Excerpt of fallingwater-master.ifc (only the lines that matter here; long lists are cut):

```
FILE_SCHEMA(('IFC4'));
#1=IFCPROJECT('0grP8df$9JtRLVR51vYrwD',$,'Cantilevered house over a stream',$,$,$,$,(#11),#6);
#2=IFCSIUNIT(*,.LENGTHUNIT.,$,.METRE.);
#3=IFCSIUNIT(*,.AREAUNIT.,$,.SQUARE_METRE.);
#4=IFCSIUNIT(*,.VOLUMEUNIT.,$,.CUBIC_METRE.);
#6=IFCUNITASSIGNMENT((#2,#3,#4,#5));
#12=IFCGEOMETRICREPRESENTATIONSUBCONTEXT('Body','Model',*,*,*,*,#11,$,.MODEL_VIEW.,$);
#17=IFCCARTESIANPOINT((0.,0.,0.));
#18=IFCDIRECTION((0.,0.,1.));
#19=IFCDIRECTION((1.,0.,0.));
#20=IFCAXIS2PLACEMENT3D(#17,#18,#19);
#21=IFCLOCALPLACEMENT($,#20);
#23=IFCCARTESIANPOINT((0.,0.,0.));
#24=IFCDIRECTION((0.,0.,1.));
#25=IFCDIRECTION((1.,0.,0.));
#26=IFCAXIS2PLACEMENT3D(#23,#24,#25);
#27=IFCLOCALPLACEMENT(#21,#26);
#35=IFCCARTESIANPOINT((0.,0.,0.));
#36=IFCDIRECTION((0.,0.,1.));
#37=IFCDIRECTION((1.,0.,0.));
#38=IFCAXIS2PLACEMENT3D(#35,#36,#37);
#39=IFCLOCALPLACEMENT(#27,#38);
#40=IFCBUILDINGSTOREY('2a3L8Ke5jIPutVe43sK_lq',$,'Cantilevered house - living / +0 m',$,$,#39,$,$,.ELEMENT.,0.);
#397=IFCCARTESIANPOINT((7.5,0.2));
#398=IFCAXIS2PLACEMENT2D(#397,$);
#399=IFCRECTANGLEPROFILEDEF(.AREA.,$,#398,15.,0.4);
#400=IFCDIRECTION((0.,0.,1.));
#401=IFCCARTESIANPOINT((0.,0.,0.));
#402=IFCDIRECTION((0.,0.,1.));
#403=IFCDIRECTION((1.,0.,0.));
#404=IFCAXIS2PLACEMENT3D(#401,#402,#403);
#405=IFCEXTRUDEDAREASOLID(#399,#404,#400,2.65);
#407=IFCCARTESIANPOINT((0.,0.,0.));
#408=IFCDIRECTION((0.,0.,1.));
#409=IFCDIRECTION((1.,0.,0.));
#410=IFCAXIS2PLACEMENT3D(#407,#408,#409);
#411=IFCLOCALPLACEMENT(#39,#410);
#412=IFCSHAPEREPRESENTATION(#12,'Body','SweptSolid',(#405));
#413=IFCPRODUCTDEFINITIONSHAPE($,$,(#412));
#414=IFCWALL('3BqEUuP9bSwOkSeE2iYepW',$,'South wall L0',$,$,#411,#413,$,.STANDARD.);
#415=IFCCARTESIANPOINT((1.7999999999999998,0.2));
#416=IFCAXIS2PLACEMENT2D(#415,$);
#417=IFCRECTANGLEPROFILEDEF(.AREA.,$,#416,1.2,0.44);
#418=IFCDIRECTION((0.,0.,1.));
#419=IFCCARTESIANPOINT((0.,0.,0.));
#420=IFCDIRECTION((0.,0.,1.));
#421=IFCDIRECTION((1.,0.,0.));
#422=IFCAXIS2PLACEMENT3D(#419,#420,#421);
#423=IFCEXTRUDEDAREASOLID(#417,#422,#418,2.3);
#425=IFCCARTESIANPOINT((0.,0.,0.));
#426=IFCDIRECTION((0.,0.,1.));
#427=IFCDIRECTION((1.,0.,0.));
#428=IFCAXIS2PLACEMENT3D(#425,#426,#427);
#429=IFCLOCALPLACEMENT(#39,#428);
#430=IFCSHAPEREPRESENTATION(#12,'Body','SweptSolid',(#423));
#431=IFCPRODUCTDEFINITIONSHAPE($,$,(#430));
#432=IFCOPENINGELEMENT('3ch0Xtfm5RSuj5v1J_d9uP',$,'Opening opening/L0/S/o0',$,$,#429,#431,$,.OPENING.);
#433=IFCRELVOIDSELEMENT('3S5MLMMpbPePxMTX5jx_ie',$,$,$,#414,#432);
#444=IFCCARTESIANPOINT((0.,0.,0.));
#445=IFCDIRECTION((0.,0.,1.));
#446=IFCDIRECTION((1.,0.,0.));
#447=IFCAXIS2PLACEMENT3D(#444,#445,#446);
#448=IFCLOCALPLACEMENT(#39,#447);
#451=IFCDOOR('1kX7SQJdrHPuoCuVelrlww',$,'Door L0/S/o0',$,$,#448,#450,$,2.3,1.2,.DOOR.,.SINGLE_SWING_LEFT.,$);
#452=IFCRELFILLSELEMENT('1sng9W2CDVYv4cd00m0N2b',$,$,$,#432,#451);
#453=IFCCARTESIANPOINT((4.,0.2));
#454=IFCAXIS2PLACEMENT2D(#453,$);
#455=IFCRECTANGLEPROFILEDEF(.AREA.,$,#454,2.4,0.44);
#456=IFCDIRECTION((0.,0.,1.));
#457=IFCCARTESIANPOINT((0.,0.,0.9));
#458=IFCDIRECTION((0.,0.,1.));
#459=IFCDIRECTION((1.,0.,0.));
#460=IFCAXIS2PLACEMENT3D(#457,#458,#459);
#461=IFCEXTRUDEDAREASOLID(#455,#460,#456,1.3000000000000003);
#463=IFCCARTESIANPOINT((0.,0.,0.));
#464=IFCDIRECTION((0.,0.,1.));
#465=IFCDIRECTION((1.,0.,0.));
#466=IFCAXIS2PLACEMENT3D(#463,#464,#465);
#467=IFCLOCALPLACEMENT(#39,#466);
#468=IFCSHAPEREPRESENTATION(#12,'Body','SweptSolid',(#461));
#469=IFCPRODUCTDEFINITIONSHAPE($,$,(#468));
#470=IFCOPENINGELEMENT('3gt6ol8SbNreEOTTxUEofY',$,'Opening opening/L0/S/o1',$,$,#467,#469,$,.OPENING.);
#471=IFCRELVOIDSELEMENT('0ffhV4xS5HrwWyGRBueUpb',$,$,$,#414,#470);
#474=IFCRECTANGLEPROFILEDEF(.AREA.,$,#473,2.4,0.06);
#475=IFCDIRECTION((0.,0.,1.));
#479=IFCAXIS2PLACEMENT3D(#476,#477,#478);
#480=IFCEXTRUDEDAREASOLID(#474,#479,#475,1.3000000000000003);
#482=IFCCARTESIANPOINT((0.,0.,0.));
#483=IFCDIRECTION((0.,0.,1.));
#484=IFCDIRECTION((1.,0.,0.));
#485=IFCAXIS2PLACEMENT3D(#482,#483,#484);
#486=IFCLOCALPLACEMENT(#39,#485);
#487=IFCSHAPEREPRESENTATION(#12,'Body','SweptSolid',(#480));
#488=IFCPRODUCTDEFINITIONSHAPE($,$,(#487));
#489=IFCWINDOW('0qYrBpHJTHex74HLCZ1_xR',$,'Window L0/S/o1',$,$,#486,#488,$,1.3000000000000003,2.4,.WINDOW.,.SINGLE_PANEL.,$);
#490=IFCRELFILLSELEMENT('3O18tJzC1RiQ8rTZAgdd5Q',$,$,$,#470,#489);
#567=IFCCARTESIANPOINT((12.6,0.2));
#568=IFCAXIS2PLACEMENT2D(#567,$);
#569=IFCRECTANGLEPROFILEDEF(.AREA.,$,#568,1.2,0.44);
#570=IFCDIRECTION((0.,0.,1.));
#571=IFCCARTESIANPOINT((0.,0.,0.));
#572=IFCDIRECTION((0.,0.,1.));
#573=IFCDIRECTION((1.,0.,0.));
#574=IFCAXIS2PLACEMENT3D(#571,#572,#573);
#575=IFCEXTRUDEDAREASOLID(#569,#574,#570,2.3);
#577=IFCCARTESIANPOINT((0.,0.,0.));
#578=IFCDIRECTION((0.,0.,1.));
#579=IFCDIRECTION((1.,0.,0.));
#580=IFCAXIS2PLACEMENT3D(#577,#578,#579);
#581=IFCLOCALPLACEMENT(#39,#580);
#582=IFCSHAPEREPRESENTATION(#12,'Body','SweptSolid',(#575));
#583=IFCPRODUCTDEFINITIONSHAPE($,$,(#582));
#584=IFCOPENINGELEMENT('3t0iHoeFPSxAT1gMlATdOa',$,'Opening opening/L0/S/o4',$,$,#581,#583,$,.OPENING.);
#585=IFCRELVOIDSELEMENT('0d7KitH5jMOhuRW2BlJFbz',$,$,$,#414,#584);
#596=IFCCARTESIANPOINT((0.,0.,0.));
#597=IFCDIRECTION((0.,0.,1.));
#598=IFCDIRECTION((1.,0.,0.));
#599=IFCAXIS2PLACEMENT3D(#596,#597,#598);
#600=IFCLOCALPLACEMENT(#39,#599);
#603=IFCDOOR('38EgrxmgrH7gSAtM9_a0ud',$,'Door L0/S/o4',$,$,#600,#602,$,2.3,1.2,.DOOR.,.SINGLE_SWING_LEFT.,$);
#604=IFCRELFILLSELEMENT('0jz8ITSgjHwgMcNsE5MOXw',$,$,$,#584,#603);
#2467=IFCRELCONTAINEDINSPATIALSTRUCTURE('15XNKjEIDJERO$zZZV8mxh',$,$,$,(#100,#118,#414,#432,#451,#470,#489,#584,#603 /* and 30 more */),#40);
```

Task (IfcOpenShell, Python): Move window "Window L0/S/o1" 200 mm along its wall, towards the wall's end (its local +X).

```python
import ifcopenshell
import ifcopenshell.api.geometry
import ifcopenshell.util.placement
import ifcopenshell.util.unit

model = ifcopenshell.open("fallingwater-master.ifc")
unit_scale = ifcopenshell.util.unit.calculate_unit_scale(model)

window = model.by_guid("0qYrBpHJTHex74HLCZ1_xR")
opening = window.FillsVoids[0].RelatingOpeningElement
wall = opening.VoidsElements[0].RelatingBuildingElement

wall_matrix = ifcopenshell.util.placement.get_local_placement(wall.ObjectPlacement)
shift = wall_matrix[:3, 0] * 0.2 / unit_scale
before = ifcopenshell.util.placement.get_local_placement(window.ObjectPlacement)[:3, 3].copy()

# The window is not placed relative to its opening, so move both.
for product in (opening, window):
    matrix = ifcopenshell.util.placement.get_local_placement(product.ObjectPlacement)
    matrix[:3, 3] += shift
    ifcopenshell.api.geometry.edit_object_placement(model, product=product, matrix=matrix, is_si=False)

after = ifcopenshell.util.placement.get_local_placement(window.ObjectPlacement)[:3, 3]
print("window moved by", (after - before).round(3) + 0.0)

model.write("fallingwater-master_v2.ifc")
```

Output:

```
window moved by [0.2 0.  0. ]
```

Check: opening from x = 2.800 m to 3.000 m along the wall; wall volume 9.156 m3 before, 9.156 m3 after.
